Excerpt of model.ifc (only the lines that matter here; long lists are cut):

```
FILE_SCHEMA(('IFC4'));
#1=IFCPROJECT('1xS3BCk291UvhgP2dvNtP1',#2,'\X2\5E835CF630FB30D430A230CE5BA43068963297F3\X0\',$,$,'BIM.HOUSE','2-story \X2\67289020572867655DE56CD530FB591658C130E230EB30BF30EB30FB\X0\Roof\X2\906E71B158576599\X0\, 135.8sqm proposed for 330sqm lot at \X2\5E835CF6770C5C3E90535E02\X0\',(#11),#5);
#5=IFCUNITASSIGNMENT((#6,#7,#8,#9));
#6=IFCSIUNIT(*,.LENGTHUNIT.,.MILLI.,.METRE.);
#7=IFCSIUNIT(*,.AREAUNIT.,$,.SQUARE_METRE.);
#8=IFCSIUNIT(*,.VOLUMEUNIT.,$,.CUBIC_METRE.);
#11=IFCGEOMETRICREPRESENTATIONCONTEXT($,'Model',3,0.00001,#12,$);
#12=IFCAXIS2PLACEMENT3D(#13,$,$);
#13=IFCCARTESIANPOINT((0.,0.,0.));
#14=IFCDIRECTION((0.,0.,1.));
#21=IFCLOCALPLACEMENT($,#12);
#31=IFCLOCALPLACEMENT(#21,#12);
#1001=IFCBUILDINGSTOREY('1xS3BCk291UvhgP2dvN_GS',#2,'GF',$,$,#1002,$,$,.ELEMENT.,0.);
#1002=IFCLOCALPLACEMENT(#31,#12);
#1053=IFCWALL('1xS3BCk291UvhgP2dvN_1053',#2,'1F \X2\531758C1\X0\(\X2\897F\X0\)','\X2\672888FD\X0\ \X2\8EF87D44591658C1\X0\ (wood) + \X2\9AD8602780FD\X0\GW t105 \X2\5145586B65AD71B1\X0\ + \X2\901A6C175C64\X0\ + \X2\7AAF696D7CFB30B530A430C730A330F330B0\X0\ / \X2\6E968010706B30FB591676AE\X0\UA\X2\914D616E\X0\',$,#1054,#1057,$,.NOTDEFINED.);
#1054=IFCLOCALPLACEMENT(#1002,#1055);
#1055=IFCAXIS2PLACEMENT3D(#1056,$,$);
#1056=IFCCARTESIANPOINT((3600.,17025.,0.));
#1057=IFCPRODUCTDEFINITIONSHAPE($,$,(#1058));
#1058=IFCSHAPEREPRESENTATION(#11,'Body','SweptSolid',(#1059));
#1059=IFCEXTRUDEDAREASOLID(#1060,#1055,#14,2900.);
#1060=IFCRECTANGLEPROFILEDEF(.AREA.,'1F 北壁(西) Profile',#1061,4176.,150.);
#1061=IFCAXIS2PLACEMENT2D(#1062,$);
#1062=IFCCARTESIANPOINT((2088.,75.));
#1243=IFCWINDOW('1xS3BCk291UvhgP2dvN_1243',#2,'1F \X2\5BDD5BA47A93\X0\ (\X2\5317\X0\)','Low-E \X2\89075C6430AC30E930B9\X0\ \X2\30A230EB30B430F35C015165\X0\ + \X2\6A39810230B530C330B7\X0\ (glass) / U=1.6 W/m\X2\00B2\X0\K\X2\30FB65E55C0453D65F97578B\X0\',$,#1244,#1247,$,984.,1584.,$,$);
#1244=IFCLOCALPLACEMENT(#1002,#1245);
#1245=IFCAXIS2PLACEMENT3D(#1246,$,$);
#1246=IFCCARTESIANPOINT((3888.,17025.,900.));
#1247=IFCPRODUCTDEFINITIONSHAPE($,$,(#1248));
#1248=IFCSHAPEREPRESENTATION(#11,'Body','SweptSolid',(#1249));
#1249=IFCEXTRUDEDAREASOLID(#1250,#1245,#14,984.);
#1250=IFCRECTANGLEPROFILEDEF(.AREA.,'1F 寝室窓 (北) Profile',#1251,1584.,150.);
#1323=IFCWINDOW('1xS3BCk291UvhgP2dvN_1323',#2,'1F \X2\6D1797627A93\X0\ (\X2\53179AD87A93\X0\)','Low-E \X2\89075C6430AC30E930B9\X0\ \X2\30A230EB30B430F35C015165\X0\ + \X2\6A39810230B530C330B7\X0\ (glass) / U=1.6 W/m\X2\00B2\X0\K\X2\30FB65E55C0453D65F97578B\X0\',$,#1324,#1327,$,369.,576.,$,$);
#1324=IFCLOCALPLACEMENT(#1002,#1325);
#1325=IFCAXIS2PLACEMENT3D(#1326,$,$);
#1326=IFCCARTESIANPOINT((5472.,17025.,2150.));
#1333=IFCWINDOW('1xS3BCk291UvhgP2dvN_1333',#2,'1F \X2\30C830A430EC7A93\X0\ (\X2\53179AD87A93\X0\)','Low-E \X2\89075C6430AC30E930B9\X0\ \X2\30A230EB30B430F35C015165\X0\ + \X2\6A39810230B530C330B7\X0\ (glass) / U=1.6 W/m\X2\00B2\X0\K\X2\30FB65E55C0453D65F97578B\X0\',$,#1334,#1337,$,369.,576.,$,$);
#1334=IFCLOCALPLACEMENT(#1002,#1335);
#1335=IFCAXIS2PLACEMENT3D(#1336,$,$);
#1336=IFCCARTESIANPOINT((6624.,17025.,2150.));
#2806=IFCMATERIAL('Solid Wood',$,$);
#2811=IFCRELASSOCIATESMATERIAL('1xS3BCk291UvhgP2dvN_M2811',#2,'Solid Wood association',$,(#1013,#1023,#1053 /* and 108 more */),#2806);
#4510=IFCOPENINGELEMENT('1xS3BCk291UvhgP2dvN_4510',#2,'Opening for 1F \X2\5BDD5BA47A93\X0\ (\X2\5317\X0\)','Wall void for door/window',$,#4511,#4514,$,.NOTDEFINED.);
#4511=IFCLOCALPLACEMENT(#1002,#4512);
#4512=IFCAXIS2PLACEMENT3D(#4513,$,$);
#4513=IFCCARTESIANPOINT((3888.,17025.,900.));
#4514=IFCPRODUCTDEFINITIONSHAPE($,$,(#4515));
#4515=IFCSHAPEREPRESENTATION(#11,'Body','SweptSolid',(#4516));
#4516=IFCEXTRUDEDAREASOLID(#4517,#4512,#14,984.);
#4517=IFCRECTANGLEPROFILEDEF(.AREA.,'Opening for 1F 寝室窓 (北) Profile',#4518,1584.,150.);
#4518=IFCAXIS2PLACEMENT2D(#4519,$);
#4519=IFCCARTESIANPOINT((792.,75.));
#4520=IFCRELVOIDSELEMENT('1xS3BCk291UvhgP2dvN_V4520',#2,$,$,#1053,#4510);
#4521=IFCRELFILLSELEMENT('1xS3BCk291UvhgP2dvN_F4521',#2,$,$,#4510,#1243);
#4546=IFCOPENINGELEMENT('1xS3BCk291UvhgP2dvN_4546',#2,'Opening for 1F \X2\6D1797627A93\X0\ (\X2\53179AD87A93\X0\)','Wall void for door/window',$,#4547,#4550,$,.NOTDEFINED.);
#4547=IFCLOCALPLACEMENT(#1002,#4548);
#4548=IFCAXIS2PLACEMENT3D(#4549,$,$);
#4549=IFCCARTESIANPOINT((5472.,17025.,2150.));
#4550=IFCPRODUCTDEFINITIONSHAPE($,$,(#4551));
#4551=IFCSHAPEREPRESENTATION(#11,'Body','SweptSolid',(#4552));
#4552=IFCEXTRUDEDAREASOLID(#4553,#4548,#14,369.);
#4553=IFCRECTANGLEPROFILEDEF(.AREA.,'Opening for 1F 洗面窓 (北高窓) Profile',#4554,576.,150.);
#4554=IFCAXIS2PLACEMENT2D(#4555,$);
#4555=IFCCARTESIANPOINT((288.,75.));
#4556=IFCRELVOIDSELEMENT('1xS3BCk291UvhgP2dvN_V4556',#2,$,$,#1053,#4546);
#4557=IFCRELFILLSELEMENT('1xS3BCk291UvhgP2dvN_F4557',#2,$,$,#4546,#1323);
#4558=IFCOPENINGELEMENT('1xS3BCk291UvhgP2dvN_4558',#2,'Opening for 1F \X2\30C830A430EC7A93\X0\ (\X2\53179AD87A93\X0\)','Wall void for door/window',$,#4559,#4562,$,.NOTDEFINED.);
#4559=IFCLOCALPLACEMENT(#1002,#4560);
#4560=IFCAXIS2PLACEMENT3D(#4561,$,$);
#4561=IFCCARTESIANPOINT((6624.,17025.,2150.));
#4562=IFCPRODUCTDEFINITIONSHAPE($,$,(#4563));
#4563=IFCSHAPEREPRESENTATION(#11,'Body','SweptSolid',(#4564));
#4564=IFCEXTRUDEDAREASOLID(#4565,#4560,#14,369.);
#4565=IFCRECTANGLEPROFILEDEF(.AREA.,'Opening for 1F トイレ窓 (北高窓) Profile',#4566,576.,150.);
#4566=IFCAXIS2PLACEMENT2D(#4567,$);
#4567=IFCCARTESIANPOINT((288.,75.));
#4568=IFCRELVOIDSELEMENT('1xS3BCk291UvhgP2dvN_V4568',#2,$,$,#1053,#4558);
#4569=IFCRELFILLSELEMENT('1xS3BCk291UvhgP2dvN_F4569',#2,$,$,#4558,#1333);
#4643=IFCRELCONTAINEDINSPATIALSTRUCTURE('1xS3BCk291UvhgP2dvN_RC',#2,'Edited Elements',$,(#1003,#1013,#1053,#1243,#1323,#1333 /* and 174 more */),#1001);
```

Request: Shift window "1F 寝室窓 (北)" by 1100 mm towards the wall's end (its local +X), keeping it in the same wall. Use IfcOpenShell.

```python
import ifcopenshell
import ifcopenshell.api.geometry
import ifcopenshell.util.placement

model = ifcopenshell.open("model.ifc")

window = model.by_guid("1xS3BCk291UvhgP2dvN_1243")
opening = window.FillsVoids[0].RelatingOpeningElement
wall = opening.VoidsElements[0].RelatingBuildingElement

wall_matrix = ifcopenshell.util.placement.get_local_placement(wall.ObjectPlacement)
shift = wall_matrix[:3, 0] * 1100.0
before = ifcopenshell.util.placement.get_local_placement(window.ObjectPlacement)[:3, 3].copy()

# The window is not placed relative to its opening, so move both.
for product in (opening, window):
    matrix = ifcopenshell.util.placement.get_local_placement(product.ObjectPlacement)
    matrix[:3, 3] += shift
    ifcopenshell.api.geometry.edit_object_placement(model, product=product, matrix=matrix, is_si=False)

after = ifcopenshell.util.placement.get_local_placement(window.ObjectPlacement)[:3, 3]
print("window moved by", (after - before).round(3) + 0.0)

model.write("model_rev.ifc")
```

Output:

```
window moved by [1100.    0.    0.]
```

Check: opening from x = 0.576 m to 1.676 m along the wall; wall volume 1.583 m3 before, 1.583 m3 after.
